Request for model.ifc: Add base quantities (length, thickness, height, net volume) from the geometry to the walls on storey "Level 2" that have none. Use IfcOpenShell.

First a look at what the model holds.

```python
import ifcopenshell
import ifcopenshell.util.element
import ifcopenshell.util.unit

model = ifcopenshell.open("model.ifc")
print(model.schema)
for unit_type in ("LENGTHUNIT", "AREAUNIT", "VOLUMEUNIT"):
    print(unit_type, ifcopenshell.util.unit.calculate_unit_scale(model, unit_type))
storey = next(s for s in model.by_type("IfcBuildingStorey") if s.Name == "Level 2")
walls = [e for e in ifcopenshell.util.element.get_decomposition(storey) if e.is_a("IfcWall")]
for e in sorted(walls, key=lambda e: e.id()):
    print(e.id(), e.is_a(), e.Name, list(ifcopenshell.util.element.get_psets(e, qtos_only=True)), sep=" | ")
```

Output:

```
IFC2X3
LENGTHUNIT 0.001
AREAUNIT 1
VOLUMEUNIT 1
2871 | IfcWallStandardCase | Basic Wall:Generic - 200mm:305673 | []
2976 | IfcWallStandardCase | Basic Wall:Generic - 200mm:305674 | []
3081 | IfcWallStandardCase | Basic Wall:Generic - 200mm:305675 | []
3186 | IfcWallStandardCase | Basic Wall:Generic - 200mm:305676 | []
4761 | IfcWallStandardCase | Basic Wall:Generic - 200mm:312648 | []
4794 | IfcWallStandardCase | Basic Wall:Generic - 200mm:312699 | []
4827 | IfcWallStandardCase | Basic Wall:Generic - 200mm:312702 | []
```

```python
import ifcopenshell
import ifcopenshell.api.pset
import ifcopenshell.geom
import ifcopenshell.util.element
import ifcopenshell.util.shape
import ifcopenshell.util.unit

model = ifcopenshell.open("model.ifc")
unit_scale = ifcopenshell.util.unit.calculate_unit_scale(model)
volume_scale = ifcopenshell.util.unit.calculate_unit_scale(model, "VOLUMEUNIT")
settings = ifcopenshell.geom.settings()

storey = next(s for s in model.by_type("IfcBuildingStorey") if s.Name == "Level 2")
walls = [e for e in ifcopenshell.util.element.get_decomposition(storey) if e.is_a("IfcWall")]

for e in sorted(walls, key=lambda e: e.id()):
    if ifcopenshell.util.element.get_psets(e, qtos_only=True, should_inherit=False):
        continue
    # Geometry comes back in metres, in the element's own axes.
    shape = ifcopenshell.geom.create_shape(settings, e)
    values = {
        "Length": ifcopenshell.util.shape.get_x(shape.geometry) / unit_scale,
        "Width": ifcopenshell.util.shape.get_y(shape.geometry) / unit_scale,
        "Height": ifcopenshell.util.shape.get_z(shape.geometry) / unit_scale,
        "NetVolume": ifcopenshell.util.shape.get_volume(shape.geometry) / volume_scale,
    }
    qto = ifcopenshell.api.pset.add_qto(model, product=e, name="BaseQuantities")
    ifcopenshell.api.pset.edit_qto(model, qto=qto, properties=values)
    print(e.id(), {k: round(v, 3) for k, v in values.items()})

model.write("model_v2.ifc")
```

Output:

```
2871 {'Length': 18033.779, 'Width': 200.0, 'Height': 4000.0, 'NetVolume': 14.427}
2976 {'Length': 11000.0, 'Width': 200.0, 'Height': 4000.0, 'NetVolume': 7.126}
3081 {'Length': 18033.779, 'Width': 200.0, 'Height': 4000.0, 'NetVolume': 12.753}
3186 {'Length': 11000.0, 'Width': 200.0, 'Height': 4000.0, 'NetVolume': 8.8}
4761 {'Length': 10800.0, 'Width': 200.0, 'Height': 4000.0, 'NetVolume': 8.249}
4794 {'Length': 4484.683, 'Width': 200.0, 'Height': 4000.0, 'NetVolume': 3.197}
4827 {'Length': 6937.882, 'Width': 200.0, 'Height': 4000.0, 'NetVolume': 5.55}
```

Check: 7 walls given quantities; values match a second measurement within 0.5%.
